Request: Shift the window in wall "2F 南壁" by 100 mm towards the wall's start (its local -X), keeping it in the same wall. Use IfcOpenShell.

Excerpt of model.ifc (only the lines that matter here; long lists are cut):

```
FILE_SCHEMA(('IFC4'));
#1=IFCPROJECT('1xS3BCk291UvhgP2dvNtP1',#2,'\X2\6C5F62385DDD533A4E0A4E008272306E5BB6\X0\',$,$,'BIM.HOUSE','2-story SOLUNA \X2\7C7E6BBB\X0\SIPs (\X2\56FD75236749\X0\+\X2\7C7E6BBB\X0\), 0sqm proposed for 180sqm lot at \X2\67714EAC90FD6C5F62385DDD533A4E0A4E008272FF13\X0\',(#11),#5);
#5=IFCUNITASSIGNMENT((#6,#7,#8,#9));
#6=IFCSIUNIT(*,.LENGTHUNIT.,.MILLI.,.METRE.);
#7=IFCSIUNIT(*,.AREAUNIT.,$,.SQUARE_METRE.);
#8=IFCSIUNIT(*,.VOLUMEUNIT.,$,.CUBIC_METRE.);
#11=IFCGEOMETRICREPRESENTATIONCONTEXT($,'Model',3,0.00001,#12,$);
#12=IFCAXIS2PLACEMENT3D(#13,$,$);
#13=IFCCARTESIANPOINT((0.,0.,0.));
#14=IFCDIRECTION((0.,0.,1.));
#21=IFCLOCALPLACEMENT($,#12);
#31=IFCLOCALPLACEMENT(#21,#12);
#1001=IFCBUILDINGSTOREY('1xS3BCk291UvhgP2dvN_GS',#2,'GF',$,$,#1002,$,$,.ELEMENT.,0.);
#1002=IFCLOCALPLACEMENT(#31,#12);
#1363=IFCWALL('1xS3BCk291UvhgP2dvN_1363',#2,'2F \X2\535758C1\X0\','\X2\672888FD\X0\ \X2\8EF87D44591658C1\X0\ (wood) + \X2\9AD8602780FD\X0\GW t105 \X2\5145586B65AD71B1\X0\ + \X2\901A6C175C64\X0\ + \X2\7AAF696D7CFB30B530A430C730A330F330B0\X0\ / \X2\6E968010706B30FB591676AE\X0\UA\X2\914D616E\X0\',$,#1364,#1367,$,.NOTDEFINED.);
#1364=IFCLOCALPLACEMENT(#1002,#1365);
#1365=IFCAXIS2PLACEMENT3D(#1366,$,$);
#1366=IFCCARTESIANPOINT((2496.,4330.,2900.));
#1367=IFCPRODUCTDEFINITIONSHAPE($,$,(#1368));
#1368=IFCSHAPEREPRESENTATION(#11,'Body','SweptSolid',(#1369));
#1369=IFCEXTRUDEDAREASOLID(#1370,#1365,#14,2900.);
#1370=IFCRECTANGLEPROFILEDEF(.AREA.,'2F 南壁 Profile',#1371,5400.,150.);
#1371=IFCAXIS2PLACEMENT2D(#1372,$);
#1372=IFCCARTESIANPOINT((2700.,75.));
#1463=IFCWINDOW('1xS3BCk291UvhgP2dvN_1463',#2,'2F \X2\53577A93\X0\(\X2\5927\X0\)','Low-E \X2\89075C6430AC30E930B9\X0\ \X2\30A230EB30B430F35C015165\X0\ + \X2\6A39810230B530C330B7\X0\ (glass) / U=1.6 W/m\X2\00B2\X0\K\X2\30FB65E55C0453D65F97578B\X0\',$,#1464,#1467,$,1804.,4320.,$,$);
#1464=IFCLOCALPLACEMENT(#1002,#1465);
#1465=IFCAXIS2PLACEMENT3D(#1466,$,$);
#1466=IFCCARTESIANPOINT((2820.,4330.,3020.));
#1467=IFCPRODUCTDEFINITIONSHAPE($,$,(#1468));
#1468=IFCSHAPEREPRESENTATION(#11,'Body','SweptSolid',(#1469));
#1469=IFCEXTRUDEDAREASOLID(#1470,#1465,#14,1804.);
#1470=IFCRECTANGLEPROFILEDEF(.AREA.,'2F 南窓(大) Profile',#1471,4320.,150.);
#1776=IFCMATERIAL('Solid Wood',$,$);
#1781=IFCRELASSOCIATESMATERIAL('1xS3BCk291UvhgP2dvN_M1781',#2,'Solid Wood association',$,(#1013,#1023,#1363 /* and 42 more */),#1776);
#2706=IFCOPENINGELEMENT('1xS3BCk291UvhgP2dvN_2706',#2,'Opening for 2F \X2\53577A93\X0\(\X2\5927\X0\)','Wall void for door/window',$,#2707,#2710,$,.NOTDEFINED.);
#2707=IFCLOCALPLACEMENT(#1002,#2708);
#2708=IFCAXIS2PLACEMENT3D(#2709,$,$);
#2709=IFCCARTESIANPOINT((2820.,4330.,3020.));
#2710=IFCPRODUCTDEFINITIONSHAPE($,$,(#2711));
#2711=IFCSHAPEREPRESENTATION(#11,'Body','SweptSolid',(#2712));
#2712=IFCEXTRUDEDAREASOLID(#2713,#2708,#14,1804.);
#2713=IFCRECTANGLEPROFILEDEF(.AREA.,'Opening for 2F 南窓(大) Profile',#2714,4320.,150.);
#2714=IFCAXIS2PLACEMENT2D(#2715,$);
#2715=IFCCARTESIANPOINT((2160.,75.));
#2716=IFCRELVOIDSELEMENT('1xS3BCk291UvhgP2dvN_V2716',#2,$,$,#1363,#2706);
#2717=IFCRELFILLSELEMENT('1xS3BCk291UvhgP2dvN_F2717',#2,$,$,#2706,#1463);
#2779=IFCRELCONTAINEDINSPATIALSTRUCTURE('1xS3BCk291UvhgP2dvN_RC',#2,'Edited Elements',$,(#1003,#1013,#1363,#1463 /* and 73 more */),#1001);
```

```python
import ifcopenshell
import ifcopenshell.api.geometry
import ifcopenshell.util.placement
import ifcopenshell.util.unit

model = ifcopenshell.open("model.ifc")
unit_scale = ifcopenshell.util.unit.calculate_unit_scale(model)

window = model.by_guid("1xS3BCk291UvhgP2dvN_1463")
opening = window.FillsVoids[0].RelatingOpeningElement
wall = opening.VoidsElements[0].RelatingBuildingElement

wall_matrix = ifcopenshell.util.placement.get_local_placement(wall.ObjectPlacement)
shift = wall_matrix[:3, 0] * -0.1 / unit_scale
before = ifcopenshell.util.placement.get_local_placement(window.ObjectPlacement)[:3, 3].copy()

# The window is not placed relative to its opening, so move both.
for product in (opening, window):
    matrix = ifcopenshell.util.placement.get_local_placement(product.ObjectPlacement)
    matrix[:3, 3] += shift
    ifcopenshell.api.geometry.edit_object_placement(model, product=product, matrix=matrix, is_si=False)

after = ifcopenshell.util.placement.get_local_placement(window.ObjectPlacement)[:3, 3]
print("window moved by", (after - before).round(3) + 0.0)

model.write("model-out.ifc")
```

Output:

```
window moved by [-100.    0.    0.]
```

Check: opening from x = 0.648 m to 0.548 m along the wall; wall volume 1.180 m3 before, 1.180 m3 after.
